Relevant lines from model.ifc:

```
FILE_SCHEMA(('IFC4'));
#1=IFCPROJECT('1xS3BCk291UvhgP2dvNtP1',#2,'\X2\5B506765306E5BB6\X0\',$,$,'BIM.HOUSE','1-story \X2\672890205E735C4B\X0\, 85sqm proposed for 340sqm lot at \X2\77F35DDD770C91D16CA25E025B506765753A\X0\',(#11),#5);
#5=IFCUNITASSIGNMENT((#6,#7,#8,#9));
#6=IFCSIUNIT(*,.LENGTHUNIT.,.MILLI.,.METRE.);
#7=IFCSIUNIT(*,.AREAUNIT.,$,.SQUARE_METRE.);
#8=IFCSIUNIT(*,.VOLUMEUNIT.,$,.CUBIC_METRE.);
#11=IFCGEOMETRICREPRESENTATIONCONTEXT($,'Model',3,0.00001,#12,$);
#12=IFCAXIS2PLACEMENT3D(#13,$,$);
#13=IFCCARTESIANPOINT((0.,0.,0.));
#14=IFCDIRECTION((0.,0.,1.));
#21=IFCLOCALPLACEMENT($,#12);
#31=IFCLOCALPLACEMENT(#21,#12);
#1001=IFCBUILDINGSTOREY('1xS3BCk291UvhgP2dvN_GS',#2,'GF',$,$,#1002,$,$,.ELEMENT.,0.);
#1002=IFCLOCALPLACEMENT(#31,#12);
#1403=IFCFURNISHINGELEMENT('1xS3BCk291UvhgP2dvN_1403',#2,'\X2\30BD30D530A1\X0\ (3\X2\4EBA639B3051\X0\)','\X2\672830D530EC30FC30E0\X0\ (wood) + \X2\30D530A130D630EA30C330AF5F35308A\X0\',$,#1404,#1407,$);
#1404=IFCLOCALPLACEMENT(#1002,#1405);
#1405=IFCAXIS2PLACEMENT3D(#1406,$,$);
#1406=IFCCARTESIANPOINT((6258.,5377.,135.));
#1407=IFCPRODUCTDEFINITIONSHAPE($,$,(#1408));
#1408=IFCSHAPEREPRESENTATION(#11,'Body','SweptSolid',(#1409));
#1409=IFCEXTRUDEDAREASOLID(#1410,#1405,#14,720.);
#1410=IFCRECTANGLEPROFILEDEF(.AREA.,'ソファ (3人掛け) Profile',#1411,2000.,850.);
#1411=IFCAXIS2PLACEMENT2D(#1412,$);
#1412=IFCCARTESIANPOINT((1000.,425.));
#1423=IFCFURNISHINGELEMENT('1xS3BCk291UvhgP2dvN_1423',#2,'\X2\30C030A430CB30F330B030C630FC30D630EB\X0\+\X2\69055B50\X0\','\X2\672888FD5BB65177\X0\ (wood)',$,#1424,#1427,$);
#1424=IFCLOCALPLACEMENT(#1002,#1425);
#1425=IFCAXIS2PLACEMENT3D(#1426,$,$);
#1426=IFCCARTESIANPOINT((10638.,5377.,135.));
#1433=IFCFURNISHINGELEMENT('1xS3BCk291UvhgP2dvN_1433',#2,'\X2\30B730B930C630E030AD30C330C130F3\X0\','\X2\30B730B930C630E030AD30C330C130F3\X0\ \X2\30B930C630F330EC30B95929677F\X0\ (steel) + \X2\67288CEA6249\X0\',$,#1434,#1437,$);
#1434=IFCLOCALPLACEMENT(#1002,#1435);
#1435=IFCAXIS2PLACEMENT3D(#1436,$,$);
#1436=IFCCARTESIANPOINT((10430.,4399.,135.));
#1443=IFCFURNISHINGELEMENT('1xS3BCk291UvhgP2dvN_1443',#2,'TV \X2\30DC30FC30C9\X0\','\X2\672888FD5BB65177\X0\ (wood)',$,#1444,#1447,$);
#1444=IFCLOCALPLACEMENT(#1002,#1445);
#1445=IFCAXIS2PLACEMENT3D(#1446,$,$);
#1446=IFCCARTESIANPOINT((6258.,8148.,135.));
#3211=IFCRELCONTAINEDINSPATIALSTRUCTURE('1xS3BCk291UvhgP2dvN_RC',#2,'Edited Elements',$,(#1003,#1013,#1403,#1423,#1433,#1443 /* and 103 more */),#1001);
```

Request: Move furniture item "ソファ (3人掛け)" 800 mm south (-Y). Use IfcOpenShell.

```python
import ifcopenshell
import ifcopenshell.api.geometry
import ifcopenshell.util.placement

model = ifcopenshell.open("model.ifc")

item = model.by_id(1403)
matrix = ifcopenshell.util.placement.get_local_placement(item.ObjectPlacement)
matrix[1, 3] -= 800.0
ifcopenshell.api.geometry.edit_object_placement(model, product=item, matrix=matrix, is_si=False)

print(ifcopenshell.util.placement.get_local_placement(item.ObjectPlacement).round(3) + 0.0)

model.write("model_rev.ifc")
```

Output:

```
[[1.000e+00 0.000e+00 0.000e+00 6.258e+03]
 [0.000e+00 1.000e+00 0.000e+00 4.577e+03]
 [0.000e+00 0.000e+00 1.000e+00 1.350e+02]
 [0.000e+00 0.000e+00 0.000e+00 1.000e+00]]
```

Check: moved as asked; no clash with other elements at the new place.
